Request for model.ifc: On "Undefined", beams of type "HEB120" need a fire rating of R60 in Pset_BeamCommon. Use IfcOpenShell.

First a look at what the model holds.

```python
import ifcopenshell
import ifcopenshell.util.element

model = ifcopenshell.open("model.ifc")
print(model.schema)
storey = next(s for s in model.by_type("IfcBuildingStorey") if s.Name == "Undefined")
beams = [e for e in ifcopenshell.util.element.get_decomposition(storey) if e.is_a("IfcBeam")]
seen = {}
for e in beams:
    element_type = ifcopenshell.util.element.get_type(e)
    key = (element_type.Name if element_type != e and element_type else None, ifcopenshell.util.element.get_pset(e, "Pset_BeamCommon", "FireRating"))
    seen[key] = seen.get(key, 0) + 1
for (name, value), count in sorted(seen.items(), key=str):
    print(count, "x", name, "|", value)
```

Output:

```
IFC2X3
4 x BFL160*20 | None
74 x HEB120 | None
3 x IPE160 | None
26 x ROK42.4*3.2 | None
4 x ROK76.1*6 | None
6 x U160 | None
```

```python
import ifcopenshell
import ifcopenshell.api.pset
import ifcopenshell.util.element

model = ifcopenshell.open("model.ifc")

storey = next(s for s in model.by_type("IfcBuildingStorey") if s.Name == "Undefined")
beams = [e for e in ifcopenshell.util.element.get_decomposition(storey) if e.is_a("IfcBeam")]

count = 0
for e in beams:
    element_type = ifcopenshell.util.element.get_type(e)
    if element_type in (None, e) or element_type.Name != "HEB120":
        continue
    # add_pset returns the element's existing set when there is one.
    pset = ifcopenshell.api.pset.add_pset(model, product=e, name="Pset_BeamCommon")
    ifcopenshell.api.pset.edit_pset(model, pset=pset, properties={"FireRating": "R60"})
    count += 1

print(count, "beams updated")

model.write("model_updated.ifc")
```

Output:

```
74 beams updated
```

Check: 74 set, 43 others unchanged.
